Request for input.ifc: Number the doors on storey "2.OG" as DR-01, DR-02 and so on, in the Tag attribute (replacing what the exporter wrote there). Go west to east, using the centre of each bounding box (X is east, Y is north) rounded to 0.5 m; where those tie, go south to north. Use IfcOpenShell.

First a look at what the model holds.

```python
import ifcopenshell
import ifcopenshell.util.element
import ifcopenshell.util.placement

model = ifcopenshell.open("input.ifc")
print(model.schema)
storey = next(s for s in model.by_type("IfcBuildingStorey") if s.Name == "2.OG")
doors = [e for e in ifcopenshell.util.element.get_decomposition(storey) if e.is_a("IfcDoor")]
for e in sorted(doors, key=lambda e: e.id()):
    origin = ifcopenshell.util.placement.get_local_placement(e.ObjectPlacement)[:3, 3]
    print(e.id(), e.Tag, e.Name, origin.round(2) + 0.0, sep=" | ")
```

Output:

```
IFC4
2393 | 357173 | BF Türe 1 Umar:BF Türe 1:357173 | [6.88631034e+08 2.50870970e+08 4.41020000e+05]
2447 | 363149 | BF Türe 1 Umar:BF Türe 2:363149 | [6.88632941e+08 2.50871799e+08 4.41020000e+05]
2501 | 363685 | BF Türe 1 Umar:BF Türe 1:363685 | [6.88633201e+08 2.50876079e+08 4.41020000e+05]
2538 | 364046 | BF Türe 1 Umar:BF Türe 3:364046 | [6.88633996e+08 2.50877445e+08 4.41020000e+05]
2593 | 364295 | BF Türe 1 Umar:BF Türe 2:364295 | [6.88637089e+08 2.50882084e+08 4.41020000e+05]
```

```python
import ifcopenshell
import ifcopenshell.geom
import ifcopenshell.util.element
import ifcopenshell.util.shape

model = ifcopenshell.open("input.ifc")
settings = ifcopenshell.geom.settings()
settings.set("use-world-coords", True)


def centre(element):
    shape = ifcopenshell.geom.create_shape(settings, element)
    return ifcopenshell.util.shape.get_bbox_centroid(shape.geometry)


storey = next(s for s in model.by_type("IfcBuildingStorey") if s.Name == "2.OG")
doors = [e for e in ifcopenshell.util.element.get_decomposition(storey) if e.is_a("IfcDoor")]

# Insertion points can sit at a corner or the storey origin, so sort by the geometry (in metres).
centres = {e: centre(e) for e in doors}
doors.sort(key=lambda e: (round(centres[e][0] / 0.5), centres[e][1]))

for i, e in enumerate(doors, start=1):
    number = f"DR-{i:02d}"
    e.Tag = number
    print(e.id(), number)

model.write("input-out.ifc")
```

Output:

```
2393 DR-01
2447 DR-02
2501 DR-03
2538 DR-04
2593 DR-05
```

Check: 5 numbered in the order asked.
